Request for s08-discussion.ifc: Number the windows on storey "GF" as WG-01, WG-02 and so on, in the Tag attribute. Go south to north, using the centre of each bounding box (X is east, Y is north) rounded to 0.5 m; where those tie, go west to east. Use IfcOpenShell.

First a look at what the model holds.

```python
import ifcopenshell
import ifcopenshell.util.element
import ifcopenshell.util.placement

model = ifcopenshell.open("s08-discussion.ifc")
print(model.schema)
storey = next(s for s in model.by_type("IfcBuildingStorey") if s.Name == "GF")
windows = [e for e in ifcopenshell.util.element.get_decomposition(storey) if e.is_a("IfcWindow")]
for e in sorted(windows, key=lambda e: e.id()):
    origin = ifcopenshell.util.placement.get_local_placement(e.ObjectPlacement)[:3, 3]
    print(e.id(), e.Tag, e.Name, origin.round(2) + 0.0, sep=" | ")
```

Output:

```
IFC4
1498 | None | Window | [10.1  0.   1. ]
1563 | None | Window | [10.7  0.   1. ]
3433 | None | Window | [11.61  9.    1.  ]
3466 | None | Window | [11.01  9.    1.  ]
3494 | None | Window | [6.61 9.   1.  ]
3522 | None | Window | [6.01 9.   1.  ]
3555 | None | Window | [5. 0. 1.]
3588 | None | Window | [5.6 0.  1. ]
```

```python
import ifcopenshell
import ifcopenshell.geom
import ifcopenshell.util.element
import ifcopenshell.util.shape

model = ifcopenshell.open("s08-discussion.ifc")
settings = ifcopenshell.geom.settings()
settings.set("use-world-coords", True)


def centre(element):
    shape = ifcopenshell.geom.create_shape(settings, element)
    return ifcopenshell.util.shape.get_bbox_centroid(shape.geometry)


storey = next(s for s in model.by_type("IfcBuildingStorey") if s.Name == "GF")
windows = [e for e in ifcopenshell.util.element.get_decomposition(storey) if e.is_a("IfcWindow")]

# Insertion points can sit at a corner or the storey origin, so sort by the geometry (in metres).
centres = {e: centre(e) for e in windows}
windows.sort(key=lambda e: (round(centres[e][1] / 0.5), centres[e][0]))

for i, e in enumerate(windows, start=1):
    number = f"WG-{i:02d}"
    e.Tag = number
    print(e.id(), number)

model.write("s08-discussion_edited.ifc")
```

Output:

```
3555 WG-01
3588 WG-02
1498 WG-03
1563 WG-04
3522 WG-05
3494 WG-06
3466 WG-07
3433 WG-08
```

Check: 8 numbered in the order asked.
